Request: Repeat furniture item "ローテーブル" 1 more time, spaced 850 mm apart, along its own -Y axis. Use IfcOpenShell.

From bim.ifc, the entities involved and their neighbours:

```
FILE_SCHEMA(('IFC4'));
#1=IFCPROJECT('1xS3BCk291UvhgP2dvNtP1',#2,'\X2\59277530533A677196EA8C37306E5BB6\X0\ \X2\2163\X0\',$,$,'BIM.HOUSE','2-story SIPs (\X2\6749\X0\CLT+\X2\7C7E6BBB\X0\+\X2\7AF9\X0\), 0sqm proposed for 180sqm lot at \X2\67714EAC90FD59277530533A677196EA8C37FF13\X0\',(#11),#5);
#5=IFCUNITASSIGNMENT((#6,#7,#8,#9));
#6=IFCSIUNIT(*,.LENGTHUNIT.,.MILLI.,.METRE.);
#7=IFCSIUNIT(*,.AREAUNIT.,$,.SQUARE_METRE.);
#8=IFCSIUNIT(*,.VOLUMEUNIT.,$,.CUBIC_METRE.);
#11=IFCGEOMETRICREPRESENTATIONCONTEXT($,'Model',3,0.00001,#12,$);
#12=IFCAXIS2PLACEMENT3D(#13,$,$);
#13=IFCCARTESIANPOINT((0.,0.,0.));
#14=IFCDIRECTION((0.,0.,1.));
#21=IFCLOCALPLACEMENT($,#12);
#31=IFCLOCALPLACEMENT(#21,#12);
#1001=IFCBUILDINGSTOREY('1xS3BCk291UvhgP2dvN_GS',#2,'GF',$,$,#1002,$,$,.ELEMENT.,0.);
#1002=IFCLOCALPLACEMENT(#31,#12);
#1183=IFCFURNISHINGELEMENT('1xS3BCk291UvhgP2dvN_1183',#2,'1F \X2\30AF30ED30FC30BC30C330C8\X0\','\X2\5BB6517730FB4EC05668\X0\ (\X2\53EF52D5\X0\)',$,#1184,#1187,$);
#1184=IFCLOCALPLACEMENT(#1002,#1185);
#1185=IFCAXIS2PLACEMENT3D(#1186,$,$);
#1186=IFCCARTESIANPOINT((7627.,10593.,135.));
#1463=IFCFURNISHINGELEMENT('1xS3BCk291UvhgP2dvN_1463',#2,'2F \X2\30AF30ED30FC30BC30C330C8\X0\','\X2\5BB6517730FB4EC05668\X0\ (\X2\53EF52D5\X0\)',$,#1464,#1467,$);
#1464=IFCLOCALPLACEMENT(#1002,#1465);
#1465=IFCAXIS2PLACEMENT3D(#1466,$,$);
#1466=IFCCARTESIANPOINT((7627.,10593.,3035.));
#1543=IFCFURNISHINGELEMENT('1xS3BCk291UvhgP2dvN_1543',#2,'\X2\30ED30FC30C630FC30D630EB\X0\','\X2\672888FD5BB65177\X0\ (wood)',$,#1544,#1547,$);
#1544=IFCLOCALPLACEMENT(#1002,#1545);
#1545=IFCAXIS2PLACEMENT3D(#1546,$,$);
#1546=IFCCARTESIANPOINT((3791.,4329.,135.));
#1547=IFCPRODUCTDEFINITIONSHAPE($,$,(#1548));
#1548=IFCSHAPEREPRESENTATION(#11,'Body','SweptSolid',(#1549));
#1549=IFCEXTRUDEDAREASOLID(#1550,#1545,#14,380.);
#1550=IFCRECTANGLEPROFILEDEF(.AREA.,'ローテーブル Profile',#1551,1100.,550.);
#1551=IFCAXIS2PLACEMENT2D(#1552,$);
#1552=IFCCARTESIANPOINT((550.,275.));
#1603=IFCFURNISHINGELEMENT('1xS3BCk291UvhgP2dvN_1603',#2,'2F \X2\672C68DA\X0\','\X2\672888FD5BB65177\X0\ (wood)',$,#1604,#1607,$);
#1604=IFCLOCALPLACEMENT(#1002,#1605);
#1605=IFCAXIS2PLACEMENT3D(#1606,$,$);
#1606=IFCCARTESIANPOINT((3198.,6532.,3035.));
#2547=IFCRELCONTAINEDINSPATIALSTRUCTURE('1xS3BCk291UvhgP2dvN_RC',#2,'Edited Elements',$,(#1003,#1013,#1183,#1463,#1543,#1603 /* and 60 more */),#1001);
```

```python
import ifcopenshell
import ifcopenshell.api.geometry
import ifcopenshell.api.root
import ifcopenshell.util.element
import ifcopenshell.util.placement
import ifcopenshell.util.unit

model = ifcopenshell.open("bim.ifc")
unit_scale = ifcopenshell.util.unit.calculate_unit_scale(model)


def reuse_history(source, copy):
    """copy_class also copies each property set's owner history, people and application; keep the originals."""
    for rel in copy.IsDefinedBy:
        if rel.is_a("IfcRelDefinesByProperties") and (history := rel.RelatingPropertyDefinition.OwnerHistory):
            rel.RelatingPropertyDefinition.OwnerHistory = source.OwnerHistory
            ifcopenshell.util.element.remove_deep2(model, history)


source = model.by_id(1543)
base = ifcopenshell.util.placement.get_local_placement(source.ObjectPlacement)
step = -base[:3, 1] * 0.85 / unit_scale

for i in range(1, 2):
    copy = ifcopenshell.api.root.copy_class(model, product=source)
    copy.Representation = ifcopenshell.util.element.copy_deep(
        model, source.Representation, exclude=["IfcGeometricRepresentationContext", "IfcRepresentationMap"]
    )
    reuse_history(source, copy)
    matrix = base.copy()
    matrix[:3, 3] += i * step
    print("added at", matrix[:3, 3].round(3) + 0.0)
    ifcopenshell.api.geometry.edit_object_placement(model, product=copy, matrix=matrix, is_si=False)

model.write("bim-out.ifc")
```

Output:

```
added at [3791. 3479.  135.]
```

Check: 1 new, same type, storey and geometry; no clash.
